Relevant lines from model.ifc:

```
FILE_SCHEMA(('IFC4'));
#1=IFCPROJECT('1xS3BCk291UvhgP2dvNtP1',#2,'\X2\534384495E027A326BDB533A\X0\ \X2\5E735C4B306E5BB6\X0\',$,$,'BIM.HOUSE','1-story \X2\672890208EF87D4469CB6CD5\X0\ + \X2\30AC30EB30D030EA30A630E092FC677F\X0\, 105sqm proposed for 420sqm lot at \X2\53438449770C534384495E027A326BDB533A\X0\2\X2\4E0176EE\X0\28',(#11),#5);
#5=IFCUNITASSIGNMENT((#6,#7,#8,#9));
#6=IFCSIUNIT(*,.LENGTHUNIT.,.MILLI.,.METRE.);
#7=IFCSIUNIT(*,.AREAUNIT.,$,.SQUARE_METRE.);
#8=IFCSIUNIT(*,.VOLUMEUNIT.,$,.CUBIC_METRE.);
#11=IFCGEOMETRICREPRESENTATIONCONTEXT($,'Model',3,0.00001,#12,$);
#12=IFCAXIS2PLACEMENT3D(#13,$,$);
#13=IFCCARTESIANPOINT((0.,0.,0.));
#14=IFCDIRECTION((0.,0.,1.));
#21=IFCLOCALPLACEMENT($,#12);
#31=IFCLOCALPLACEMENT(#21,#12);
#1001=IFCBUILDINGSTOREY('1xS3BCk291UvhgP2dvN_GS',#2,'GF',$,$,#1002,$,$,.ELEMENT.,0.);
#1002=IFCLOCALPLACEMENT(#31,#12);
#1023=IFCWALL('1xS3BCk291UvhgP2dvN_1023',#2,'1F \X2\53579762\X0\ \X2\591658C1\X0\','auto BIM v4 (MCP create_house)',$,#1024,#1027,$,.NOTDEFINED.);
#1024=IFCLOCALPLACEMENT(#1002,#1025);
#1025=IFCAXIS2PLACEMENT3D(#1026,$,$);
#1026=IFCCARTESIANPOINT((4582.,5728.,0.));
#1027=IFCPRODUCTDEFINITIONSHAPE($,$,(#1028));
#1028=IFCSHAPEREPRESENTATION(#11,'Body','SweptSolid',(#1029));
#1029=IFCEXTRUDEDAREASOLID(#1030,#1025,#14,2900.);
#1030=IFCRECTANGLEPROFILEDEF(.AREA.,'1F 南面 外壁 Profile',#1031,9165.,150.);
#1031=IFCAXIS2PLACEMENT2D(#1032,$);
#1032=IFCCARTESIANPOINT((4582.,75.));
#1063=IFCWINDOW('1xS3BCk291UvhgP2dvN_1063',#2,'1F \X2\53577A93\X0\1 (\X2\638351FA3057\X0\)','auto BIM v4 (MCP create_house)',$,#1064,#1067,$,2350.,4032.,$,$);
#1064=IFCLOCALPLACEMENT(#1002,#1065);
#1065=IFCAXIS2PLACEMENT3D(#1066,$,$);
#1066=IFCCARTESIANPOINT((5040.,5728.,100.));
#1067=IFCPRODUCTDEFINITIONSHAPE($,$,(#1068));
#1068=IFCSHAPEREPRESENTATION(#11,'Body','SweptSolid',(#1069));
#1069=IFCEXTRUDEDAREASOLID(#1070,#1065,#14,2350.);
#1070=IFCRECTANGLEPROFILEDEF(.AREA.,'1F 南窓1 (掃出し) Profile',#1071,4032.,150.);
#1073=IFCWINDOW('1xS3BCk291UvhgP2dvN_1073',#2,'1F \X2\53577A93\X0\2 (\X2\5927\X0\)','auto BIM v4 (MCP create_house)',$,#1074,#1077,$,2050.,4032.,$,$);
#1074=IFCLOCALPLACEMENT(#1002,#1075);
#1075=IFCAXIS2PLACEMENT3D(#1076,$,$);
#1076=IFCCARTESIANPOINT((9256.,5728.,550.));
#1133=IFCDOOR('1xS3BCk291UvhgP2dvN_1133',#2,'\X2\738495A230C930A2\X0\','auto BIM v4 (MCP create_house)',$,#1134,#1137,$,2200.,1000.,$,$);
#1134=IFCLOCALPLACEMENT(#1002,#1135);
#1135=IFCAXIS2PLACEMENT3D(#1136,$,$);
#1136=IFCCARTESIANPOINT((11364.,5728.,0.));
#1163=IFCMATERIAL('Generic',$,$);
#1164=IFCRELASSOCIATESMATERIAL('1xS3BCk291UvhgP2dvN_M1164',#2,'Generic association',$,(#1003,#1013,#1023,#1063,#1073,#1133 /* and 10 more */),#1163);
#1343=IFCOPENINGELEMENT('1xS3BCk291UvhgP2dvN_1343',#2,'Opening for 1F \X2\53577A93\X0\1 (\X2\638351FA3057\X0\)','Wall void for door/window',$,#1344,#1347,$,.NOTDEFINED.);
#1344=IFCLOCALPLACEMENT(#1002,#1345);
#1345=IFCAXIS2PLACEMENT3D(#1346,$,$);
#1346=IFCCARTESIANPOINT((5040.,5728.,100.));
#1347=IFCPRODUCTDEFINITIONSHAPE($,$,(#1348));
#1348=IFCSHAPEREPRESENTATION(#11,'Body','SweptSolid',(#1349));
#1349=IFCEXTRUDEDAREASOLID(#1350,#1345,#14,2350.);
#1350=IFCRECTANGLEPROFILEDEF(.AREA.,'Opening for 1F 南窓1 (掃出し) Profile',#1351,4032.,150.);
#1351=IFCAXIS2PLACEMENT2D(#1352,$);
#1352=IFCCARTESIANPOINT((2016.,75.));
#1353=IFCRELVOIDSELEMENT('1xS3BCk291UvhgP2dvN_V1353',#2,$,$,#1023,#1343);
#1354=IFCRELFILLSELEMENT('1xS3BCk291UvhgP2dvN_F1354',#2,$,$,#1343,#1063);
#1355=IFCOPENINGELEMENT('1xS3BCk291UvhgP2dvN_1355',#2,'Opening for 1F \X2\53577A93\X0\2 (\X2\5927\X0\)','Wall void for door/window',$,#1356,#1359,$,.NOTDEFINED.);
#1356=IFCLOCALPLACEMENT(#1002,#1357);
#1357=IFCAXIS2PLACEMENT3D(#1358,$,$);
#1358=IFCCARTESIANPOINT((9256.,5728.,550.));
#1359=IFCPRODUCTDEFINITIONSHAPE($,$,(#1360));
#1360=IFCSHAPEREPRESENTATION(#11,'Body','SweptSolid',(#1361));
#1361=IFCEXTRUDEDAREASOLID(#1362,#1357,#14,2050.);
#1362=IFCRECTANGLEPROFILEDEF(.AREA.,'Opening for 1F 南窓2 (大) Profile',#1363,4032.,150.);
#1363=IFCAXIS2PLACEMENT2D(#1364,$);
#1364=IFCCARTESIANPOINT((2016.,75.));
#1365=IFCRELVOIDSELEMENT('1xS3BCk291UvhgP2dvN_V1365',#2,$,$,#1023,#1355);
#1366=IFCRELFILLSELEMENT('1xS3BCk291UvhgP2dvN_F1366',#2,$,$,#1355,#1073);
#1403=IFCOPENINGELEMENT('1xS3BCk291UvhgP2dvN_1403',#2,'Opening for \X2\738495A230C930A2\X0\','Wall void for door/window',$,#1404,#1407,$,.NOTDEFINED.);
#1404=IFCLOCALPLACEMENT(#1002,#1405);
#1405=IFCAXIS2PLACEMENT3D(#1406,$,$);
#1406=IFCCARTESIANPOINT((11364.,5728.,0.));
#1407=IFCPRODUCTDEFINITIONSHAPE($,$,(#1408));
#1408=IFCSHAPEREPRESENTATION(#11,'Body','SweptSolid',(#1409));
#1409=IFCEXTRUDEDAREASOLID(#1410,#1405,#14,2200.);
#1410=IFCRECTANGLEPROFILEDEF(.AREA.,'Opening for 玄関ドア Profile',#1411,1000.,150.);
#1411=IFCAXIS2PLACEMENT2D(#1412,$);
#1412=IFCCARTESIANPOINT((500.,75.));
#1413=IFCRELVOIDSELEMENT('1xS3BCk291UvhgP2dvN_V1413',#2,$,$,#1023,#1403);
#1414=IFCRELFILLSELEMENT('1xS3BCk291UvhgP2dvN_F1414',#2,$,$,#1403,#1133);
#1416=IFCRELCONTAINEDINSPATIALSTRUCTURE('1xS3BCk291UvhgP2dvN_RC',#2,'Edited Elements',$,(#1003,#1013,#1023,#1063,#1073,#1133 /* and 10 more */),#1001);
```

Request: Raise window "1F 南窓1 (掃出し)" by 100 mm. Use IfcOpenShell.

```python
import numpy as np
import ifcopenshell
import ifcopenshell.api.geometry
import ifcopenshell.util.placement
import ifcopenshell.util.unit

model = ifcopenshell.open("model.ifc")
unit_scale = ifcopenshell.util.unit.calculate_unit_scale(model)

window = model.by_guid("1xS3BCk291UvhgP2dvN_1063")
opening = window.FillsVoids[0].RelatingOpeningElement
dz = 0.1 / unit_scale

shift = np.array([0.0, 0.0, dz])
# The window is not placed relative to its opening, so move both.
for product in (opening, window):
    matrix = ifcopenshell.util.placement.get_local_placement(product.ObjectPlacement)
    matrix[:3, 3] += shift
    ifcopenshell.api.geometry.edit_object_placement(model, product=product, matrix=matrix, is_si=False)

print(f"moved by {dz * unit_scale:+.3f} m")

model.write("model_rev.ifc")
```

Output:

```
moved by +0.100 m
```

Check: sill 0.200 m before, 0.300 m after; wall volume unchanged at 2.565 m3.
